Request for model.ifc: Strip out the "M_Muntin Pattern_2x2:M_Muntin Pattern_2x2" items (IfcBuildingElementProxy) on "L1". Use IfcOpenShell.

First a look at what the model holds.

```python
import ifcopenshell
import ifcopenshell.util.element

model = ifcopenshell.open("model.ifc")
print(model.schema)
storey = next(s for s in model.by_type("IfcBuildingStorey") if s.Name == "L1")
proxies = [e for e in ifcopenshell.util.element.get_decomposition(storey) if e.is_a("IfcBuildingElementProxy")]
seen = {}
for e in proxies:
    element_type = ifcopenshell.util.element.get_type(e)
    name = element_type.Name if element_type not in (None, e) else None
    seen[name] = seen.get(name, 0) + 1
for name, count in sorted(seen.items(), key=str):
    print(count, "x", name)
```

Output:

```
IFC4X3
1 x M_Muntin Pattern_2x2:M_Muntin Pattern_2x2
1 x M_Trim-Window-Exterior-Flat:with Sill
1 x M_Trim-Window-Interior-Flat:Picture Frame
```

```python
import ifcopenshell
import ifcopenshell.api.root
import ifcopenshell.util.element

model = ifcopenshell.open("model.ifc")

storey = next(s for s in model.by_type("IfcBuildingStorey") if s.Name == "L1")
proxies = [e for e in ifcopenshell.util.element.get_decomposition(storey) if e.is_a("IfcBuildingElementProxy")]
targets = [e for e in proxies if (t := ifcopenshell.util.element.get_type(e)) not in (None, e) and t.Name == "M_Muntin Pattern_2x2:M_Muntin Pattern_2x2"]

for e in targets:
    ifcopenshell.api.root.remove_product(model, product=e)
print(len(targets), "removed")

model.write("model_updated.ifc")
```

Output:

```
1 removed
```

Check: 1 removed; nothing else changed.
